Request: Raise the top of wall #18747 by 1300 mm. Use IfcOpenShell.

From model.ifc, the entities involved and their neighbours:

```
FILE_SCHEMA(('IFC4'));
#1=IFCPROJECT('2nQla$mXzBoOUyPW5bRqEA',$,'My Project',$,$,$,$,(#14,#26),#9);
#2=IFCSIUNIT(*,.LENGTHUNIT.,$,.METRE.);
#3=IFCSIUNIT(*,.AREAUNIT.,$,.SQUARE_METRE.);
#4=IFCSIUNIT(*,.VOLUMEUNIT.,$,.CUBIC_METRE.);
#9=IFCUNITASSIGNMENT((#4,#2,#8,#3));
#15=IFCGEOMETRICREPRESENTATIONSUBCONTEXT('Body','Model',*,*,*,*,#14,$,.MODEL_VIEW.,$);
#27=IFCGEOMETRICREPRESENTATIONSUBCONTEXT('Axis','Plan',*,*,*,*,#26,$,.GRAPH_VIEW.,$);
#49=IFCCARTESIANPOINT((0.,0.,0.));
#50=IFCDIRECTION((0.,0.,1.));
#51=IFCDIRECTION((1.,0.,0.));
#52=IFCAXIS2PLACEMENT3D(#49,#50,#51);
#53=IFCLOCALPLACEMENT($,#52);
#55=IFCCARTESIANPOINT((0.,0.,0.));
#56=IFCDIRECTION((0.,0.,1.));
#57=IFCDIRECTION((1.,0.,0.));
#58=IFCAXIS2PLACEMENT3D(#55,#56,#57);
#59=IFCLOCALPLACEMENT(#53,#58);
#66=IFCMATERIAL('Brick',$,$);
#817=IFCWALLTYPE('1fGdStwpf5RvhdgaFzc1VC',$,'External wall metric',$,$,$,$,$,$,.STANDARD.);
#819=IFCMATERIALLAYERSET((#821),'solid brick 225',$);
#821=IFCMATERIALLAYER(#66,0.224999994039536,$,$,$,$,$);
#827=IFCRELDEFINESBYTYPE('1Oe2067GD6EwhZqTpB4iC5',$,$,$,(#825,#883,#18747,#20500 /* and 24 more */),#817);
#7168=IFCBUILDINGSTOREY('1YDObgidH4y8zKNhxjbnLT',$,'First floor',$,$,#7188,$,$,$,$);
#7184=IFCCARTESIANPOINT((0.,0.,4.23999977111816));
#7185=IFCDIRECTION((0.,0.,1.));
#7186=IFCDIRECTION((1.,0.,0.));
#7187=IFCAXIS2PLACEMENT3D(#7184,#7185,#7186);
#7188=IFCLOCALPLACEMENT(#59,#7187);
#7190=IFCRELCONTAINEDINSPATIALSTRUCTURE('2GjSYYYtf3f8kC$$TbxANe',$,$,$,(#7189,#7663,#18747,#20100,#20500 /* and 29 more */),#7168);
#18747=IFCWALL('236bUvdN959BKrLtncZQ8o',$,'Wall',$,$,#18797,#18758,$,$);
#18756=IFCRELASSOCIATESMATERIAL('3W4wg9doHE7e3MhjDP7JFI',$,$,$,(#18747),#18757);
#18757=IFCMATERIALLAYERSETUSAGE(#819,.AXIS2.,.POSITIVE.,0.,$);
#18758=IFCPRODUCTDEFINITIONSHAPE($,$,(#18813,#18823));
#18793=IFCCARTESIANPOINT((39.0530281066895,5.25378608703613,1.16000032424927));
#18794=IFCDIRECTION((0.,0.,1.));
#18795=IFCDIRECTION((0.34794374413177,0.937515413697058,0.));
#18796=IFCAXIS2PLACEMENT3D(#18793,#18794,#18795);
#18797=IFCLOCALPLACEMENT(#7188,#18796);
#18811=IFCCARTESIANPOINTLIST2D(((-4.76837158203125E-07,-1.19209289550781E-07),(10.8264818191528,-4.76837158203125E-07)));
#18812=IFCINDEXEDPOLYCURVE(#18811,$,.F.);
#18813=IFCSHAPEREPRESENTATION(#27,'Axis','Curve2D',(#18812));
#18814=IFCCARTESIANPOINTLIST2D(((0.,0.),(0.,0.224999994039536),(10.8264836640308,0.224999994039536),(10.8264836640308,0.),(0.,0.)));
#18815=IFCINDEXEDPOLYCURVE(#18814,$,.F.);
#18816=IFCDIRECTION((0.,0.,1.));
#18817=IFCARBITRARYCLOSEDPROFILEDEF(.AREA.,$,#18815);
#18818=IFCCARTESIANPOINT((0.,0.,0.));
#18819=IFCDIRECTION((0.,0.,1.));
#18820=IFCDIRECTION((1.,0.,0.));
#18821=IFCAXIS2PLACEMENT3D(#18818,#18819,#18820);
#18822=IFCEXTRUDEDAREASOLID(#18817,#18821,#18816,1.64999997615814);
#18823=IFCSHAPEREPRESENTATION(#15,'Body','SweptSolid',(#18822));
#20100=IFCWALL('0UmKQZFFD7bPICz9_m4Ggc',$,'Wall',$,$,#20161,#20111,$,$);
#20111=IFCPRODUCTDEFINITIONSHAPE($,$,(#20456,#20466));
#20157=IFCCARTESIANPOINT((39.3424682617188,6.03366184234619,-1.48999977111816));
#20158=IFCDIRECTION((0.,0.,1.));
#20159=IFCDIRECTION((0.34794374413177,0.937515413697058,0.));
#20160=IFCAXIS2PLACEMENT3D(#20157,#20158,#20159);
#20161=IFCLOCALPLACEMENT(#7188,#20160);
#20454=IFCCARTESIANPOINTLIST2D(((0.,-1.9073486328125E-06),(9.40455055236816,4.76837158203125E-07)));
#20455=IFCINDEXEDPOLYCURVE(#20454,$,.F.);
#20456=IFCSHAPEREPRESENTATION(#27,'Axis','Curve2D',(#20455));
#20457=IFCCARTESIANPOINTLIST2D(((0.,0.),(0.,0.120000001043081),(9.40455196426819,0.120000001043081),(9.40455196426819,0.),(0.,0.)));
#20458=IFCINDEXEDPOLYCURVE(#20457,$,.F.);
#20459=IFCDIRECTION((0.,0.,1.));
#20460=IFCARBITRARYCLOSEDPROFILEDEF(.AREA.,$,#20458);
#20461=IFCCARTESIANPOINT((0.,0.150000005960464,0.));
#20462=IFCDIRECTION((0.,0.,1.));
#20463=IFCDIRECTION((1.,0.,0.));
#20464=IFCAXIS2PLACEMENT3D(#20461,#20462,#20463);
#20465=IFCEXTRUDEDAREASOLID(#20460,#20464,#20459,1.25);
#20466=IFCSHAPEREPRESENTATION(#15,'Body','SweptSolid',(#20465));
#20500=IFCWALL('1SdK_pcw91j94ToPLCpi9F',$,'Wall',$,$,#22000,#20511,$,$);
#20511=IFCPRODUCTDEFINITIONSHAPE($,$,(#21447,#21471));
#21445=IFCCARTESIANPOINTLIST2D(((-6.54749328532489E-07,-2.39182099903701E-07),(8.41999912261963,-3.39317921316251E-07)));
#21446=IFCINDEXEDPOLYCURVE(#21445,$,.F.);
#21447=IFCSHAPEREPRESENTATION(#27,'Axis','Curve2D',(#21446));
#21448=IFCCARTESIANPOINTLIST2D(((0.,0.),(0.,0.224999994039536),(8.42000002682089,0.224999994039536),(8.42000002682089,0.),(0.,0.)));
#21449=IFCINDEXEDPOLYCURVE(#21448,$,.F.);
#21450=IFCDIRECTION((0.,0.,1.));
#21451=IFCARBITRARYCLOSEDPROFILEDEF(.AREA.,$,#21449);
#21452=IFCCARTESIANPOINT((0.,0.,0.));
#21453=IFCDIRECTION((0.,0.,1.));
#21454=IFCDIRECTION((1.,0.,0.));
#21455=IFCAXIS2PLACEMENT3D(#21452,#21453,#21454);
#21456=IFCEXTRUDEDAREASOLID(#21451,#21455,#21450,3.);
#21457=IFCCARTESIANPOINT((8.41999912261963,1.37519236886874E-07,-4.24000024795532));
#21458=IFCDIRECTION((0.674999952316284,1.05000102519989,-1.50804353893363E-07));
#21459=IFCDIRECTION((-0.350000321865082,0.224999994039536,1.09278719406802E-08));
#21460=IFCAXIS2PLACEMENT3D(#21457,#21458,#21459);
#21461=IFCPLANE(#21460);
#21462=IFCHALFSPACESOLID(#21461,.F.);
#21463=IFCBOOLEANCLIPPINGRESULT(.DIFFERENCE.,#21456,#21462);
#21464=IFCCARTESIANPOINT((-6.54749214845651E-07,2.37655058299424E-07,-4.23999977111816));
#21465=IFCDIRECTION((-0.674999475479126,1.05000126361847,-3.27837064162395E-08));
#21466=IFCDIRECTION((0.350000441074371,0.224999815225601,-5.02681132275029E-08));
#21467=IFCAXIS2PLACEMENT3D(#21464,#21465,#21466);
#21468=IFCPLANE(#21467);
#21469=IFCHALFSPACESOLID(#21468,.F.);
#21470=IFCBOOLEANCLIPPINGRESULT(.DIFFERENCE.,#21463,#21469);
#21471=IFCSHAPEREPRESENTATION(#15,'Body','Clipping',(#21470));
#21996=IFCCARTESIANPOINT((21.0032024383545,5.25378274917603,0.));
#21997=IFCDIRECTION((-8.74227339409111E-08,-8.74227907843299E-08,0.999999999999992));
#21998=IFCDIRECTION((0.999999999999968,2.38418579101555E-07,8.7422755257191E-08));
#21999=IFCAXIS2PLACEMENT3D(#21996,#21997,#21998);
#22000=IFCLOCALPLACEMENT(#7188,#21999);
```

```python
import ifcopenshell
import ifcopenshell.geom
import ifcopenshell.util.representation
import ifcopenshell.util.shape
import ifcopenshell.util.unit

model = ifcopenshell.open("model.ifc")
unit_scale = ifcopenshell.util.unit.calculate_unit_scale(model)
settings = ifcopenshell.geom.settings()


def volume(element):
    """Net volume in cubic metres, openings subtracted."""
    shape = ifcopenshell.geom.create_shape(settings, element)
    return ifcopenshell.util.shape.get_volume(shape.geometry)


wall = model.by_guid("236bUvdN959BKrLtncZQ8o")
before = volume(wall)

body = ifcopenshell.util.representation.get_representation(wall, "Model", "Body")
solid = body.Items[0]
old_height = solid.Depth
solid.Depth += 1.3 / unit_scale
after = volume(wall)

print(f"height {old_height:g} -> {solid.Depth:g}, volume {before:.3f} -> {after:.3f} m3")

model.write("model_edited.ifc")
```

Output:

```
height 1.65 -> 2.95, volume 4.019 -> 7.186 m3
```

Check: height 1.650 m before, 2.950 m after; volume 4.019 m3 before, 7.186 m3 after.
